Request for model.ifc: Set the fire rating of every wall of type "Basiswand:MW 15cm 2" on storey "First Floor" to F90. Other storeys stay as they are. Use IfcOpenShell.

First a look at what the model holds.

```python
import ifcopenshell
import ifcopenshell.util.element

model = ifcopenshell.open("model.ifc")
print(model.schema)
storey = next(s for s in model.by_type("IfcBuildingStorey") if s.Name == "First Floor")
walls = [e for e in ifcopenshell.util.element.get_decomposition(storey) if e.is_a("IfcWall")]
seen = {}
for e in walls:
    element_type = ifcopenshell.util.element.get_type(e)
    key = (element_type.Name if element_type != e and element_type else None, ifcopenshell.util.element.get_pset(e, "Pset_WallCommon", "FireRating"))
    seen[key] = seen.get(key, 0) + 1
for (name, value), count in sorted(seen.items(), key=str):
    print(count, "x", name, "|", value)
```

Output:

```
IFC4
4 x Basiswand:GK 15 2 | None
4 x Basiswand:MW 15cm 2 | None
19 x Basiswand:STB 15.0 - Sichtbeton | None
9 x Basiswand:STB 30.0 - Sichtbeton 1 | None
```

```python
import ifcopenshell
import ifcopenshell.api.pset
import ifcopenshell.util.element

model = ifcopenshell.open("model.ifc")

storey = next(s for s in model.by_type("IfcBuildingStorey") if s.Name == "First Floor")
walls = [e for e in ifcopenshell.util.element.get_decomposition(storey) if e.is_a("IfcWall")]

count = 0
for e in walls:
    element_type = ifcopenshell.util.element.get_type(e)
    if element_type in (None, e) or element_type.Name != "Basiswand:MW 15cm 2":
        continue
    # add_pset returns the element's existing set when there is one.
    pset = ifcopenshell.api.pset.add_pset(model, product=e, name="Pset_WallCommon")
    ifcopenshell.api.pset.edit_pset(model, pset=pset, properties={"FireRating": "F90"})
    count += 1

print(count, "walls updated")

model.write("model_updated.ifc")
```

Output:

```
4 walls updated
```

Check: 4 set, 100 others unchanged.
